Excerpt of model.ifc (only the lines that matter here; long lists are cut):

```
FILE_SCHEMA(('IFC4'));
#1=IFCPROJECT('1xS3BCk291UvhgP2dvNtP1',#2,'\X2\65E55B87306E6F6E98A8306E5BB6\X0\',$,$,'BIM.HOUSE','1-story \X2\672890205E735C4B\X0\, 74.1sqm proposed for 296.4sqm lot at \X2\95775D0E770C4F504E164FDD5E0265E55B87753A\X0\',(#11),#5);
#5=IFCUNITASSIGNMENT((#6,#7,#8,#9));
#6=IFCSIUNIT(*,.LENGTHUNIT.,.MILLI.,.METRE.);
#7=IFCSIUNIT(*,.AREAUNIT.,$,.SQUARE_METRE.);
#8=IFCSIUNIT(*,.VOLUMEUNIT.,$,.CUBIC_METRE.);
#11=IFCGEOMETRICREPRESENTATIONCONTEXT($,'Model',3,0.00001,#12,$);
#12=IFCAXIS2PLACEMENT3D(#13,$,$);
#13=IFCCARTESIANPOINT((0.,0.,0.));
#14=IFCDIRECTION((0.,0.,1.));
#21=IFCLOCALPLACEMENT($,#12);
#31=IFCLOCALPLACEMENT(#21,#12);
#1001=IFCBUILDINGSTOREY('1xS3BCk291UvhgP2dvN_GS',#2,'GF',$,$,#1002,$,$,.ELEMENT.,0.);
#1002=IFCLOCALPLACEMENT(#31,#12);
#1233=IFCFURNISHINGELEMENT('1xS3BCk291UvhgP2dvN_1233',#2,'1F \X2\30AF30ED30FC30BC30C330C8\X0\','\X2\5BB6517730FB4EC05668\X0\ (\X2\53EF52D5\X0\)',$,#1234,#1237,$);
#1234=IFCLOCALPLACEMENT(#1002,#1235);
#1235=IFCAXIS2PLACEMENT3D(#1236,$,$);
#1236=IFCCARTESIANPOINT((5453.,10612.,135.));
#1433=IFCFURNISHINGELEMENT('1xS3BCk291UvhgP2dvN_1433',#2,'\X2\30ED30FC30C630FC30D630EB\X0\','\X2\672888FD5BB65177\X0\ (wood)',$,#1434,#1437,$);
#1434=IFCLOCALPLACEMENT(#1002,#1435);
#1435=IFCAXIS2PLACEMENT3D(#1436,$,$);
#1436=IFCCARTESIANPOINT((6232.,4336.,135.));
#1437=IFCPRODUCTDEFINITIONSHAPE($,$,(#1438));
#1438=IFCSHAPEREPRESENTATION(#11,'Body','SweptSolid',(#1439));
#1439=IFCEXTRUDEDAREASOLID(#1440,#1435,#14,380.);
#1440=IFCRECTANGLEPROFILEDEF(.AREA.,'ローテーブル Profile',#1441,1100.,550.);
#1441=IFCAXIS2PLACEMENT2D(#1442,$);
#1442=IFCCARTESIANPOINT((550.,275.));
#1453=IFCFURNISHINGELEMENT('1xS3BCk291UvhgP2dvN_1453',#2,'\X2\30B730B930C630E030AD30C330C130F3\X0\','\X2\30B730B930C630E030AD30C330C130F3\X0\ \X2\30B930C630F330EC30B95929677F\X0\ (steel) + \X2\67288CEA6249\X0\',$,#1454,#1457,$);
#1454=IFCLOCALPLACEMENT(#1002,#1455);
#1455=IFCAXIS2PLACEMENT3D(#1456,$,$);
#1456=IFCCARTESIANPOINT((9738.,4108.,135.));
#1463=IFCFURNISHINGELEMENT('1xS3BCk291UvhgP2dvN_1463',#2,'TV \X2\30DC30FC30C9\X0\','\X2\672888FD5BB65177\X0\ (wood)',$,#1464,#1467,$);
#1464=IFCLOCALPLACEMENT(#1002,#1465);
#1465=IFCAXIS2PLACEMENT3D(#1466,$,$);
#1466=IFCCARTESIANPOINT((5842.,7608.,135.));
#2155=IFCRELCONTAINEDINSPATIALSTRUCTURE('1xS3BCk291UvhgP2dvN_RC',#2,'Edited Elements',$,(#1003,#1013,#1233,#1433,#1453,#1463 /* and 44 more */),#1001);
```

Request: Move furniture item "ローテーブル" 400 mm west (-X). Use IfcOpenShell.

```python
import ifcopenshell
import ifcopenshell.api.geometry
import ifcopenshell.util.placement
import ifcopenshell.util.unit

model = ifcopenshell.open("model.ifc")
unit_scale = ifcopenshell.util.unit.calculate_unit_scale(model)

item = model.by_id(1433)
matrix = ifcopenshell.util.placement.get_local_placement(item.ObjectPlacement)
matrix[0, 3] -= 0.4 / unit_scale
ifcopenshell.api.geometry.edit_object_placement(model, product=item, matrix=matrix, is_si=False)

print(ifcopenshell.util.placement.get_local_placement(item.ObjectPlacement).round(3) + 0.0)

model.write("model_rev.ifc")
```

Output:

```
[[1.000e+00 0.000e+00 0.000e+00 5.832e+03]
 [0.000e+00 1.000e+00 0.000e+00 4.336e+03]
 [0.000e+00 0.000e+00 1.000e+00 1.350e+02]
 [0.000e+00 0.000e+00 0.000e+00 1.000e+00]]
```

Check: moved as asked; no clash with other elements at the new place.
